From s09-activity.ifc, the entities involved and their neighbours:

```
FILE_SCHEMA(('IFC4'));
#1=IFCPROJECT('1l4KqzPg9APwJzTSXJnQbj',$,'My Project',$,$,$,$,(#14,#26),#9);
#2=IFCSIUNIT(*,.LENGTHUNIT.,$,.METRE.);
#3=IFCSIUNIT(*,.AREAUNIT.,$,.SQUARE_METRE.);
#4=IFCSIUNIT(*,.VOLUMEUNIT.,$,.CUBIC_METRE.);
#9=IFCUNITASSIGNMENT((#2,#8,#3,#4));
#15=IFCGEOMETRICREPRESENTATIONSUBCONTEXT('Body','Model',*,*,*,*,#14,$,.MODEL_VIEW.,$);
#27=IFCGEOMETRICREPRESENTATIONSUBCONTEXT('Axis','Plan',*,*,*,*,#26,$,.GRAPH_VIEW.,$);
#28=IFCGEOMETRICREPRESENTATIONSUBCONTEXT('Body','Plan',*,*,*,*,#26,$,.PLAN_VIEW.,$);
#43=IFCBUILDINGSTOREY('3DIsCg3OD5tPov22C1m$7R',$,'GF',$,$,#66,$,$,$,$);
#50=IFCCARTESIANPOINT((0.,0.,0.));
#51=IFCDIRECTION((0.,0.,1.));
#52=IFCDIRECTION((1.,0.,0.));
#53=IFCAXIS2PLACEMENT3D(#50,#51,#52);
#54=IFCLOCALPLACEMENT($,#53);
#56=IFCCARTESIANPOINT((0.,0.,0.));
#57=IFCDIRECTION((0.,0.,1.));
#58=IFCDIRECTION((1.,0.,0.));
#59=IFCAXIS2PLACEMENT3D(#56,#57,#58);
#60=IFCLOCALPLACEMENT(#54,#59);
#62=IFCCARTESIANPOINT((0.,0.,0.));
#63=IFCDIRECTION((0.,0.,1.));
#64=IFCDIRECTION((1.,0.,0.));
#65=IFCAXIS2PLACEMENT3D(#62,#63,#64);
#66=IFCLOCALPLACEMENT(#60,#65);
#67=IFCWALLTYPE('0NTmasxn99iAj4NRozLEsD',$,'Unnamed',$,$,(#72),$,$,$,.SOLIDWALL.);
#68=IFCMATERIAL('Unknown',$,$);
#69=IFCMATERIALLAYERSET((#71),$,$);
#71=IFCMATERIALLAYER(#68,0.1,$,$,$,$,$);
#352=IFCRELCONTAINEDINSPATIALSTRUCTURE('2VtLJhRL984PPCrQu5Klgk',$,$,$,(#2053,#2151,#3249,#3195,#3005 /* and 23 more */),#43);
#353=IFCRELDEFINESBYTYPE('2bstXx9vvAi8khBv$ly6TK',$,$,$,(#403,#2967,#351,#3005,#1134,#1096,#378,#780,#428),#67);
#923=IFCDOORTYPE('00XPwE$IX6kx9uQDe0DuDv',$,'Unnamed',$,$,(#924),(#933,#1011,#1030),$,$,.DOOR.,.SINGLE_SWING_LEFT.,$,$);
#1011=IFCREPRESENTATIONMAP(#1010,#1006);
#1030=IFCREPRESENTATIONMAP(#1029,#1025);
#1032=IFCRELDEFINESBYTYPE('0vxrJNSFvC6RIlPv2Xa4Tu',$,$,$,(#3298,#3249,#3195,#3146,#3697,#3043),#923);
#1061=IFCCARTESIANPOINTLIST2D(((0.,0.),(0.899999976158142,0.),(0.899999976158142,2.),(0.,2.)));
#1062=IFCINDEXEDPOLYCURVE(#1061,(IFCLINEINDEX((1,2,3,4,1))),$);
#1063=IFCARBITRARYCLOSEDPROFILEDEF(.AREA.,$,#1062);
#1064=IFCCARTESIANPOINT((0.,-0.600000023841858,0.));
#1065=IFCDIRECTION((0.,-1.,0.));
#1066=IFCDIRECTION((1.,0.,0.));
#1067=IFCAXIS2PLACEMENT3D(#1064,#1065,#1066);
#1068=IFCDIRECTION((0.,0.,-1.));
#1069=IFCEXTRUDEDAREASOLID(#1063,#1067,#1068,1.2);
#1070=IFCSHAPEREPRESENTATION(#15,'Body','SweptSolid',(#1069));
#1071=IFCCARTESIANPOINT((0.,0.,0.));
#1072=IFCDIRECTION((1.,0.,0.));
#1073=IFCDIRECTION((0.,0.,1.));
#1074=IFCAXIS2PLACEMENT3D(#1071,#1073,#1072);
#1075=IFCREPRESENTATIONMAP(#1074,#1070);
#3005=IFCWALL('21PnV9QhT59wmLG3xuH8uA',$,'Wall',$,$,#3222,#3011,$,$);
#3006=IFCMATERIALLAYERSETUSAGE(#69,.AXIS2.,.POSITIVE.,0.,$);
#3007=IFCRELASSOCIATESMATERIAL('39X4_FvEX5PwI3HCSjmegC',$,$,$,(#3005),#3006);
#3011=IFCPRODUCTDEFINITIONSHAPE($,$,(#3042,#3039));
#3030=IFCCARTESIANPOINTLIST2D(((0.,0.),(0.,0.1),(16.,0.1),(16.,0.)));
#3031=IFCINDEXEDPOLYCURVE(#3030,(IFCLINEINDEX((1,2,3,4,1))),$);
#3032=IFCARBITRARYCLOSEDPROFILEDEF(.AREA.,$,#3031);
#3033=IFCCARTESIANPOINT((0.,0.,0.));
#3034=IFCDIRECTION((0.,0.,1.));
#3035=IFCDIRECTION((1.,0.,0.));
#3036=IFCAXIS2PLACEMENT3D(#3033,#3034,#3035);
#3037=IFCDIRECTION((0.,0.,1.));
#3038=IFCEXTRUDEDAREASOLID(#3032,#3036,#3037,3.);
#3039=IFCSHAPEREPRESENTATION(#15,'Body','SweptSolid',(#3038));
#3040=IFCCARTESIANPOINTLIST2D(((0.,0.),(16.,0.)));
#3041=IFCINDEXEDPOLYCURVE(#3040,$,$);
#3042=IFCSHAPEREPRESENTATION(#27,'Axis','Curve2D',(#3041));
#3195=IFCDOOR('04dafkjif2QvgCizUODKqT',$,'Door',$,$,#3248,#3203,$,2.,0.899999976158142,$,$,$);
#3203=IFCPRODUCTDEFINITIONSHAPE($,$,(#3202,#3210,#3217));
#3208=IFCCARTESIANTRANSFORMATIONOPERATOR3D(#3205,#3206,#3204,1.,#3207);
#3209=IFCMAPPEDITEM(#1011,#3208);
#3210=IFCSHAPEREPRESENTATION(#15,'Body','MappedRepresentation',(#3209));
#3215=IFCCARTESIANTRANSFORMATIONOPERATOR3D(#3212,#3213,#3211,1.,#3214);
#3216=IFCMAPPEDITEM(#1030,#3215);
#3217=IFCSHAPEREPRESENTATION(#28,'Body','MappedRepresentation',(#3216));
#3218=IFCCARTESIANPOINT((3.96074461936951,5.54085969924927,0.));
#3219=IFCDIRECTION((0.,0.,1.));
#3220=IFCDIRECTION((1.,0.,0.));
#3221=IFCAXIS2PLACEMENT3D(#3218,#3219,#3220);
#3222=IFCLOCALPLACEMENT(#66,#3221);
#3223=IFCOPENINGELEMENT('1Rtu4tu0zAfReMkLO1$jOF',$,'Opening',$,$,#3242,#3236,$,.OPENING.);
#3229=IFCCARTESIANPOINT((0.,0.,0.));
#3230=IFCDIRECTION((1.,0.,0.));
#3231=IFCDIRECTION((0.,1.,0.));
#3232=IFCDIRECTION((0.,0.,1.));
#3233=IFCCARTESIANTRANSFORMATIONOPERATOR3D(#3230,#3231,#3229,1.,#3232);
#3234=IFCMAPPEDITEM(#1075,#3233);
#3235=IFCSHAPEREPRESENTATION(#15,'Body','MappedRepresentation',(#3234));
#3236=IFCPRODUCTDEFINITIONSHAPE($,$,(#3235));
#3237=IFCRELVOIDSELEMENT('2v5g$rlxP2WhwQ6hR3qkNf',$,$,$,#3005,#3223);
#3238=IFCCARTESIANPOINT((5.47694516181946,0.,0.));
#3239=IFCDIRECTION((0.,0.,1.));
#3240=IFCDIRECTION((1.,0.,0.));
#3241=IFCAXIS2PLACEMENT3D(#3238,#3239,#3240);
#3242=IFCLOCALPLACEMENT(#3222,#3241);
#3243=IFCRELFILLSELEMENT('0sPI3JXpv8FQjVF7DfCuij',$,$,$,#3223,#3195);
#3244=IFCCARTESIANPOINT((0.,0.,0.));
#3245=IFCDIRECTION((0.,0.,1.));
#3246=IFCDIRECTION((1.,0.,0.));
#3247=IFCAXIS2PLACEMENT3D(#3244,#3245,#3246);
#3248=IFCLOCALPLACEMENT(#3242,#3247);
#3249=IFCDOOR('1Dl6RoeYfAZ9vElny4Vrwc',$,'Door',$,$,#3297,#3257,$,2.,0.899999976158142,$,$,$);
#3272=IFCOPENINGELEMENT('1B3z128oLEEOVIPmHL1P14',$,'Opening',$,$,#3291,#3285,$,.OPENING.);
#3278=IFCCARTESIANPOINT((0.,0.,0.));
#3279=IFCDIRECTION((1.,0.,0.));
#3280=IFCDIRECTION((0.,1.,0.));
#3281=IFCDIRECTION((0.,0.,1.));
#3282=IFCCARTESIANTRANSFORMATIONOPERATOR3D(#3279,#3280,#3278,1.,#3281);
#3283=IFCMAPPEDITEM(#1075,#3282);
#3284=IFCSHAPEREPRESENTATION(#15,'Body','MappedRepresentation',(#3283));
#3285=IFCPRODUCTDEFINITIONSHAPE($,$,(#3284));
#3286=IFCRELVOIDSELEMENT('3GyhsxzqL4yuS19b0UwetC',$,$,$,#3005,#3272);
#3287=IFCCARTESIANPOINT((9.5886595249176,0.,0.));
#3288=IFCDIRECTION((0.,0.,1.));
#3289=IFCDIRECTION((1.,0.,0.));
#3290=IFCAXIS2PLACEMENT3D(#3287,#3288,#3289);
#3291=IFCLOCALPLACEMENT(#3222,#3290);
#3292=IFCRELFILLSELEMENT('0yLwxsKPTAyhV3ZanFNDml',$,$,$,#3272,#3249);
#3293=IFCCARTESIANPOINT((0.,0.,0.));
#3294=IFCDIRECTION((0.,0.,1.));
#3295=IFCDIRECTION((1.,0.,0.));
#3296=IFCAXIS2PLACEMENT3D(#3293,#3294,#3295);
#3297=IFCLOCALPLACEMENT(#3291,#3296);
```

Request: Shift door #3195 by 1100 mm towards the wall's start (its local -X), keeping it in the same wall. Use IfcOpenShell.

```python
import ifcopenshell
import ifcopenshell.api.geometry
import ifcopenshell.util.placement

model = ifcopenshell.open("s09-activity.ifc")

door = model.by_guid("04dafkjif2QvgCizUODKqT")
opening = door.FillsVoids[0].RelatingOpeningElement
wall = opening.VoidsElements[0].RelatingBuildingElement

wall_matrix = ifcopenshell.util.placement.get_local_placement(wall.ObjectPlacement)
shift = wall_matrix[:3, 0] * -1.1
before = ifcopenshell.util.placement.get_local_placement(door.ObjectPlacement)[:3, 3].copy()

# The door is placed relative to its opening, so it follows when the opening moves.
matrix = ifcopenshell.util.placement.get_local_placement(opening.ObjectPlacement)
matrix[:3, 3] += shift
ifcopenshell.api.geometry.edit_object_placement(
    model, product=opening, matrix=matrix, is_si=False, should_transform_children=True
)

after = ifcopenshell.util.placement.get_local_placement(door.ObjectPlacement)[:3, 3]
print("door moved by", (after - before).round(3) + 0.0)

model.write("s09-activity_rev.ifc")
```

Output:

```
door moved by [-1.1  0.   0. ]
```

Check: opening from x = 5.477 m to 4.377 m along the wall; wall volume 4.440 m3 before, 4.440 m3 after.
